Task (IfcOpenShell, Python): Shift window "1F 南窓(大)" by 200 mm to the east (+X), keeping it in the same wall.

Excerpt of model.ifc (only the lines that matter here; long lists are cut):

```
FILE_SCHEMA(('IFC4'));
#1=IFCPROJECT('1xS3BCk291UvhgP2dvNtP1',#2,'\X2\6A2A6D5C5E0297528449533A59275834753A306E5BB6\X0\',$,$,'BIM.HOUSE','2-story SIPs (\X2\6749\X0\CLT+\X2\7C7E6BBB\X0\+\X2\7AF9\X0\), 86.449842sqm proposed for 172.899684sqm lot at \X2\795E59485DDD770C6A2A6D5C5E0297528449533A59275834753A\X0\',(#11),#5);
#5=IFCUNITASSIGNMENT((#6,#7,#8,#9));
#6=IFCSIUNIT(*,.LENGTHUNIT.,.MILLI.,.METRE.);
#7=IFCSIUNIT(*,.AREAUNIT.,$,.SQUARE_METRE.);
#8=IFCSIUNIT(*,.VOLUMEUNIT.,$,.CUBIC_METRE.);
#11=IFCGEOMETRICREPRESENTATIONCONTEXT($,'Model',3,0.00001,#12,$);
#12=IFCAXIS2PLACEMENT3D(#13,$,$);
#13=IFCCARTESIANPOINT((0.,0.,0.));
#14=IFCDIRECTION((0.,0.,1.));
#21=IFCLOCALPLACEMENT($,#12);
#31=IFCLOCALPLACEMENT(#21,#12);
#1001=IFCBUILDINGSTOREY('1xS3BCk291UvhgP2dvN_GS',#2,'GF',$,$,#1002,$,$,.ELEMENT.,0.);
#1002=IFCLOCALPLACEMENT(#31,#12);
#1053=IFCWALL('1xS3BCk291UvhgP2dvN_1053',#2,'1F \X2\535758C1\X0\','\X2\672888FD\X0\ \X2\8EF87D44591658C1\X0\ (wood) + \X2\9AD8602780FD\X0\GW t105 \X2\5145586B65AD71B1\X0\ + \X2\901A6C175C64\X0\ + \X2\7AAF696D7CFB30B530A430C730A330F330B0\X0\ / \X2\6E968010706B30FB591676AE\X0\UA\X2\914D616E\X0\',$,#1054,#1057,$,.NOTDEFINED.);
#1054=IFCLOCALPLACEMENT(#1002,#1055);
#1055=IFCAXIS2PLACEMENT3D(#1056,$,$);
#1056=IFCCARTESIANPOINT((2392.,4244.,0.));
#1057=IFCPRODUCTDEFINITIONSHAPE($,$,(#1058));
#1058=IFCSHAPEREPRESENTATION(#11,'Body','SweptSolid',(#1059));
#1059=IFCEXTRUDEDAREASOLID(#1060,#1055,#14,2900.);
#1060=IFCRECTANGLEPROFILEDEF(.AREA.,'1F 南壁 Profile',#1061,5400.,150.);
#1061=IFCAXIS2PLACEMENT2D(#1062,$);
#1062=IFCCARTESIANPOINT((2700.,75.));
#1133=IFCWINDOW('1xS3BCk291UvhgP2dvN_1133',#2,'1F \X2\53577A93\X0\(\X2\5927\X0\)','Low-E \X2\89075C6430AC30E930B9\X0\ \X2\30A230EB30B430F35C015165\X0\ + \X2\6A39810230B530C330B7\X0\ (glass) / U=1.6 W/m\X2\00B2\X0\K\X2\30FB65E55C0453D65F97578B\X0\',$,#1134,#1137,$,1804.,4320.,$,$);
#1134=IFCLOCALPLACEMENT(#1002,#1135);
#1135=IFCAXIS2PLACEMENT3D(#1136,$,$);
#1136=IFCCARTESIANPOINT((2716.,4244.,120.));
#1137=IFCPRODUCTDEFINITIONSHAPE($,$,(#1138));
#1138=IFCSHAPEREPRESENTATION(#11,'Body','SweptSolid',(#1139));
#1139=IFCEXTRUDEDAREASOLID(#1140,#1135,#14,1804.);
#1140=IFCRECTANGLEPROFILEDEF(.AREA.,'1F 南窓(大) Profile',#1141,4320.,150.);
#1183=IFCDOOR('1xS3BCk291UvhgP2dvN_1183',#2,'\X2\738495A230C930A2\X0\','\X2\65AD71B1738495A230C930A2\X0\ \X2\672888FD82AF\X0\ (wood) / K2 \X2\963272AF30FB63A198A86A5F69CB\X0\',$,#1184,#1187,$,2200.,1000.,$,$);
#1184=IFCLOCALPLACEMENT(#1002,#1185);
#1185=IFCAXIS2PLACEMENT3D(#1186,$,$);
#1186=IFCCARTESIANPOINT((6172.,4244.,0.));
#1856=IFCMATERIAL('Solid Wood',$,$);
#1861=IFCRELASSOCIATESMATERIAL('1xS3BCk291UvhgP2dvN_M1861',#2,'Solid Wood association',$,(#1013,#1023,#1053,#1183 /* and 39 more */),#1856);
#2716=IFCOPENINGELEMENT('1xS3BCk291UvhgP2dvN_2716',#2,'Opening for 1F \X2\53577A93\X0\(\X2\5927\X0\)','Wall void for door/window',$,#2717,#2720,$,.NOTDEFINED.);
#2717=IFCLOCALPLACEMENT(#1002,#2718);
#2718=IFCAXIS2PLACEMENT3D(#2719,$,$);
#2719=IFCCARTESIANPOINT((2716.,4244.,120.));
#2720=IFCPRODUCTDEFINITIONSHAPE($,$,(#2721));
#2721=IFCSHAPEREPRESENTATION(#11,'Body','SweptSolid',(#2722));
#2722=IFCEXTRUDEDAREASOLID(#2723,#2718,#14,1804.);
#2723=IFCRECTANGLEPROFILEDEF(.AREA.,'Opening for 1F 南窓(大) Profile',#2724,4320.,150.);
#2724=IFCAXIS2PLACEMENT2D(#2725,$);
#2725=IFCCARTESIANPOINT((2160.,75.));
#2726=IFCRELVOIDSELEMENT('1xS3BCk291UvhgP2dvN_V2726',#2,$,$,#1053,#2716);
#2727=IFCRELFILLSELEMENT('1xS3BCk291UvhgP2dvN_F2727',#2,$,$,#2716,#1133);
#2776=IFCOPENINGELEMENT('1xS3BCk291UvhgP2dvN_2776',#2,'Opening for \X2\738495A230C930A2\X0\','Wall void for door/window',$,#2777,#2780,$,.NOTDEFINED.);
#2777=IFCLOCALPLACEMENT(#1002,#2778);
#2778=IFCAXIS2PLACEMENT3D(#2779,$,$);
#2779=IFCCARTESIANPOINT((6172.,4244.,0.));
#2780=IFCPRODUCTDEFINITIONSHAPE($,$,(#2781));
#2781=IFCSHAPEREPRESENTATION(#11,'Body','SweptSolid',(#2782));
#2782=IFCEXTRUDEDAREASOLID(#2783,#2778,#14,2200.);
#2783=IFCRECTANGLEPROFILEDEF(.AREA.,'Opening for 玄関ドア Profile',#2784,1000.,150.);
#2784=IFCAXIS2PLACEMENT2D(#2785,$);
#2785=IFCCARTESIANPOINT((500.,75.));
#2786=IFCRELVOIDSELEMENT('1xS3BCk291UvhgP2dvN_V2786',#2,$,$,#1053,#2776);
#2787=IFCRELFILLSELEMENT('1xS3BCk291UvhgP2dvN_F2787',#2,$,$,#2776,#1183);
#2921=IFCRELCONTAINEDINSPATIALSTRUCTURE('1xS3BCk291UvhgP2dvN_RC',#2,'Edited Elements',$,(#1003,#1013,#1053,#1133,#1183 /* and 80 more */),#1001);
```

```python
import ifcopenshell
import ifcopenshell.api.geometry
import ifcopenshell.util.placement

model = ifcopenshell.open("model.ifc")

window = model.by_guid("1xS3BCk291UvhgP2dvN_1133")
opening = window.FillsVoids[0].RelatingOpeningElement
wall = opening.VoidsElements[0].RelatingBuildingElement

wall_matrix = ifcopenshell.util.placement.get_local_placement(wall.ObjectPlacement)
shift = wall_matrix[:3, 0] * 200.0
before = ifcopenshell.util.placement.get_local_placement(window.ObjectPlacement)[:3, 3].copy()

# The window is not placed relative to its opening, so move both.
for product in (opening, window):
    matrix = ifcopenshell.util.placement.get_local_placement(product.ObjectPlacement)
    matrix[:3, 3] += shift
    ifcopenshell.api.geometry.edit_object_placement(model, product=product, matrix=matrix, is_si=False)

after = ifcopenshell.util.placement.get_local_placement(window.ObjectPlacement)[:3, 3]
print("window moved by", (after - before).round(3) + 0.0)

model.write("model_rev.ifc")
```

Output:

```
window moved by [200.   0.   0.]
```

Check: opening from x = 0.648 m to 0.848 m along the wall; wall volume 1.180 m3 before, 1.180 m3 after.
